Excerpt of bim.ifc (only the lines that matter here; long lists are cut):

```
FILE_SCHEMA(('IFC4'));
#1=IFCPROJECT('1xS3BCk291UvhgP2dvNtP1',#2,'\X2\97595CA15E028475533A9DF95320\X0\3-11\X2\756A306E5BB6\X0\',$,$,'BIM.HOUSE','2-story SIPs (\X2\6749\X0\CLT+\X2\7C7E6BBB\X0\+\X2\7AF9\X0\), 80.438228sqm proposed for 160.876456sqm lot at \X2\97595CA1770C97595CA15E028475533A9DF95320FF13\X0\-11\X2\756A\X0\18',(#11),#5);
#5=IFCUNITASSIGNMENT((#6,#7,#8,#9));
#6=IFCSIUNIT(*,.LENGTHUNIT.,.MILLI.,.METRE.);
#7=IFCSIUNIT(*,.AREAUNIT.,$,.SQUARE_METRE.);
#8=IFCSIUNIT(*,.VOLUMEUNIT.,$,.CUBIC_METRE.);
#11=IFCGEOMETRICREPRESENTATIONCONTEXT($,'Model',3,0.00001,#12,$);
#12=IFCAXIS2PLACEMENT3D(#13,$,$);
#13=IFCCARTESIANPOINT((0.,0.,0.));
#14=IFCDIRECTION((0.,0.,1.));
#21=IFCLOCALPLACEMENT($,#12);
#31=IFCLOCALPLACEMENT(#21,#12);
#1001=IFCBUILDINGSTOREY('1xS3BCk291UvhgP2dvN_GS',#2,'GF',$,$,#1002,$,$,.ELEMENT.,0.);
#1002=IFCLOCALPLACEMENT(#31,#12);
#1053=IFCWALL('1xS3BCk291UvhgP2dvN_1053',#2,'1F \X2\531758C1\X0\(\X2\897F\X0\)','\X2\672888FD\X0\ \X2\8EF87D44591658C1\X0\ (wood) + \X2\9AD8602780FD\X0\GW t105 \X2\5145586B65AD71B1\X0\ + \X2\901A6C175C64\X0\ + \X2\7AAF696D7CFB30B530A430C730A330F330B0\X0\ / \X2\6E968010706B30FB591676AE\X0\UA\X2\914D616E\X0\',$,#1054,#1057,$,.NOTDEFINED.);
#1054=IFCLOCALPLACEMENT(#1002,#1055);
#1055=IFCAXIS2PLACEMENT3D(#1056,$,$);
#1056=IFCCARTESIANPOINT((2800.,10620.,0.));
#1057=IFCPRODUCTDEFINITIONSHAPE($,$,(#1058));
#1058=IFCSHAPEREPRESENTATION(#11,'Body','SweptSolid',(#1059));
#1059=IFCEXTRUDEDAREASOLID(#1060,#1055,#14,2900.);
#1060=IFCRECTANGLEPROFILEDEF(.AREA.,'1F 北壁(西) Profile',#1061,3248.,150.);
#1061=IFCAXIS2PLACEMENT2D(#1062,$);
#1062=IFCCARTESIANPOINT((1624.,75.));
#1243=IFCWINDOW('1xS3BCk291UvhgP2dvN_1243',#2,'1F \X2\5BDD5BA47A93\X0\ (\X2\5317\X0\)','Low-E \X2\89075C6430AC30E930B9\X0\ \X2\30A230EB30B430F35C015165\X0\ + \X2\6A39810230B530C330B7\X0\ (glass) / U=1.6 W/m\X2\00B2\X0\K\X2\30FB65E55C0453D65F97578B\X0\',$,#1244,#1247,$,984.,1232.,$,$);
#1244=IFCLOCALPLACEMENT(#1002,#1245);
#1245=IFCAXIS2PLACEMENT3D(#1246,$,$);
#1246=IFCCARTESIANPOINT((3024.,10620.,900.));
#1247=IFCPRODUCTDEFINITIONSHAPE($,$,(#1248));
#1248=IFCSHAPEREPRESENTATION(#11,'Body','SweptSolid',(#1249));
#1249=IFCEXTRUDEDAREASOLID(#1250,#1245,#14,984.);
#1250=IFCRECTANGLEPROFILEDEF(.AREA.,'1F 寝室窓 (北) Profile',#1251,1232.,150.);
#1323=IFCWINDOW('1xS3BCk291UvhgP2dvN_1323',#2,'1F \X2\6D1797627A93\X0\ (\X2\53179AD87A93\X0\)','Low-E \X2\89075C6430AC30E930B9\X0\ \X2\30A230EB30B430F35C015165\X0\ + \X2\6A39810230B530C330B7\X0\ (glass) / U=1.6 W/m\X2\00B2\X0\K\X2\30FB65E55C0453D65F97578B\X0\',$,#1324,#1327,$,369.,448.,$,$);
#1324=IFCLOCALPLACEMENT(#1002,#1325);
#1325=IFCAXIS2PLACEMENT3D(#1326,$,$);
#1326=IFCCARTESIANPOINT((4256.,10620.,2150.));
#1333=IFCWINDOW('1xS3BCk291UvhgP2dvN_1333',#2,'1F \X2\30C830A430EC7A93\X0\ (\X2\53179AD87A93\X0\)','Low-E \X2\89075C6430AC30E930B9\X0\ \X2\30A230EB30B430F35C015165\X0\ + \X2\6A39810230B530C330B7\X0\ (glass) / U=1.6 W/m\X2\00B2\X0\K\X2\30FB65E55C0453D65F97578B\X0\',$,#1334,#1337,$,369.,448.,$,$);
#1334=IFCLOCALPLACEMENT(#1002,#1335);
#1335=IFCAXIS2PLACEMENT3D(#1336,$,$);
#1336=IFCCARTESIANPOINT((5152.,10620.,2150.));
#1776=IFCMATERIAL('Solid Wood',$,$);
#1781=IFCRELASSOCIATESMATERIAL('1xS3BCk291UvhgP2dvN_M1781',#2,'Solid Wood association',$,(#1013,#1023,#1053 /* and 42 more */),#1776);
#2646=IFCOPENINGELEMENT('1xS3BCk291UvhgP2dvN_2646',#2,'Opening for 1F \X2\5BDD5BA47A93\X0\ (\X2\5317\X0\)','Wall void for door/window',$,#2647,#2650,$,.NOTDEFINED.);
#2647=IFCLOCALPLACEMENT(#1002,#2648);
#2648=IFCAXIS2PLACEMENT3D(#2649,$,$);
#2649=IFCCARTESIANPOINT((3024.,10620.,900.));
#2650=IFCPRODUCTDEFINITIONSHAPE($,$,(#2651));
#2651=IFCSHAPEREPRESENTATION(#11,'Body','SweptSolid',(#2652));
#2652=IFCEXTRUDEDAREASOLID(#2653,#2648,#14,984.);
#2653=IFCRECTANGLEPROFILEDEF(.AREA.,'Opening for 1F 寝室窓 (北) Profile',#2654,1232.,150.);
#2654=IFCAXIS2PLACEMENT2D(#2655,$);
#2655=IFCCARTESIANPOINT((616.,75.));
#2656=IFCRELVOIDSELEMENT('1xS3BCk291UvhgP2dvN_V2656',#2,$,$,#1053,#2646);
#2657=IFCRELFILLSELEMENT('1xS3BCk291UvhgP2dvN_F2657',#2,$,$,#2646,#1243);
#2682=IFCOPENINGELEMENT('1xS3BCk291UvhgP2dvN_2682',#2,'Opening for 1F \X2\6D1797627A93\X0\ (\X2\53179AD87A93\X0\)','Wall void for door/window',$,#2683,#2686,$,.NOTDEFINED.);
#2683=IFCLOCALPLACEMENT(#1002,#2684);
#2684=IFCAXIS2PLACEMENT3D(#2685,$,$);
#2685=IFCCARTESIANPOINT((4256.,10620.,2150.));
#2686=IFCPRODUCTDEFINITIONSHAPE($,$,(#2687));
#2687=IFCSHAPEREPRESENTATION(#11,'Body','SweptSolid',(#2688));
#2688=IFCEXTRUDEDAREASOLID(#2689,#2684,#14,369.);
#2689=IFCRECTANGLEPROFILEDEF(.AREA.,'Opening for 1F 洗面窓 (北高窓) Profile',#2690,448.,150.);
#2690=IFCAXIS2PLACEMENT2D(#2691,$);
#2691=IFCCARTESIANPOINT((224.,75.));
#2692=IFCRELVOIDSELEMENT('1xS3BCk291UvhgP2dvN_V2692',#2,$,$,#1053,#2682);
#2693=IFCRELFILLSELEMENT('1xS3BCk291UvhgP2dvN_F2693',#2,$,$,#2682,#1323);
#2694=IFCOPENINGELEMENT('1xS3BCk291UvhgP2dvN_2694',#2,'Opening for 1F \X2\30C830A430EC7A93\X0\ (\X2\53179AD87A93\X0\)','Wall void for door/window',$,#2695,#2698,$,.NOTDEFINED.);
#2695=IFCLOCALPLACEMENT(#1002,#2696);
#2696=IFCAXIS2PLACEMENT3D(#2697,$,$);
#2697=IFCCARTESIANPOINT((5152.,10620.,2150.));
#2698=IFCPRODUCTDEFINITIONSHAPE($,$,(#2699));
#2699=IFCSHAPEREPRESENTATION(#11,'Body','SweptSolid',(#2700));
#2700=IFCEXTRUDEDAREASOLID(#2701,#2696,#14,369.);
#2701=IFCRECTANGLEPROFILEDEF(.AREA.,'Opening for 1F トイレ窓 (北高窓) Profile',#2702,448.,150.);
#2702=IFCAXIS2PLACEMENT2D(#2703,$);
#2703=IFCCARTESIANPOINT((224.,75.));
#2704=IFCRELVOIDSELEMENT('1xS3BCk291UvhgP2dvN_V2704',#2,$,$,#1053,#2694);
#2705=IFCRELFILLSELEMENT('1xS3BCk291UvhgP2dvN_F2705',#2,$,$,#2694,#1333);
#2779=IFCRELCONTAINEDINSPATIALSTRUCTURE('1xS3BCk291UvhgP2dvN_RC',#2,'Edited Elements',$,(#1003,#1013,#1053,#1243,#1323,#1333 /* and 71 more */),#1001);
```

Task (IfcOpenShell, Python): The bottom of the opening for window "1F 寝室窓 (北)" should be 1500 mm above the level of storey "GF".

```python
import numpy as np
import ifcopenshell
import ifcopenshell.api.geometry
import ifcopenshell.geom
import ifcopenshell.util.element
import ifcopenshell.util.placement
import ifcopenshell.util.shape
import ifcopenshell.util.unit

model = ifcopenshell.open("bim.ifc")
unit_scale = ifcopenshell.util.unit.calculate_unit_scale(model)

window = model.by_id(1243)
opening = window.FillsVoids[0].RelatingOpeningElement
storey = ifcopenshell.util.element.get_container(window, ifc_class="IfcBuildingStorey")
level = ifcopenshell.util.placement.get_local_placement(storey.ObjectPlacement)[2, 3]

# The opening's origin need not be at the sill, so measure its lowest point.
shape = ifcopenshell.geom.create_shape(ifcopenshell.geom.settings(), opening)
bottom = ifcopenshell.util.shape.get_shape_bottom_elevation(shape, shape.geometry) / unit_scale
dz = level + 1.5 / unit_scale - bottom

shift = np.array([0.0, 0.0, dz])
# The window is not placed relative to its opening, so move both.
for product in (opening, window):
    matrix = ifcopenshell.util.placement.get_local_placement(product.ObjectPlacement)
    matrix[:3, 3] += shift
    ifcopenshell.api.geometry.edit_object_placement(model, product=product, matrix=matrix, is_si=False)

print(f"moved by {dz * unit_scale:+.3f} m")

model.write("bim_rev.ifc")
```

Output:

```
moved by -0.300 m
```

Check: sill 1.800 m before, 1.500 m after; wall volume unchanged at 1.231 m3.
